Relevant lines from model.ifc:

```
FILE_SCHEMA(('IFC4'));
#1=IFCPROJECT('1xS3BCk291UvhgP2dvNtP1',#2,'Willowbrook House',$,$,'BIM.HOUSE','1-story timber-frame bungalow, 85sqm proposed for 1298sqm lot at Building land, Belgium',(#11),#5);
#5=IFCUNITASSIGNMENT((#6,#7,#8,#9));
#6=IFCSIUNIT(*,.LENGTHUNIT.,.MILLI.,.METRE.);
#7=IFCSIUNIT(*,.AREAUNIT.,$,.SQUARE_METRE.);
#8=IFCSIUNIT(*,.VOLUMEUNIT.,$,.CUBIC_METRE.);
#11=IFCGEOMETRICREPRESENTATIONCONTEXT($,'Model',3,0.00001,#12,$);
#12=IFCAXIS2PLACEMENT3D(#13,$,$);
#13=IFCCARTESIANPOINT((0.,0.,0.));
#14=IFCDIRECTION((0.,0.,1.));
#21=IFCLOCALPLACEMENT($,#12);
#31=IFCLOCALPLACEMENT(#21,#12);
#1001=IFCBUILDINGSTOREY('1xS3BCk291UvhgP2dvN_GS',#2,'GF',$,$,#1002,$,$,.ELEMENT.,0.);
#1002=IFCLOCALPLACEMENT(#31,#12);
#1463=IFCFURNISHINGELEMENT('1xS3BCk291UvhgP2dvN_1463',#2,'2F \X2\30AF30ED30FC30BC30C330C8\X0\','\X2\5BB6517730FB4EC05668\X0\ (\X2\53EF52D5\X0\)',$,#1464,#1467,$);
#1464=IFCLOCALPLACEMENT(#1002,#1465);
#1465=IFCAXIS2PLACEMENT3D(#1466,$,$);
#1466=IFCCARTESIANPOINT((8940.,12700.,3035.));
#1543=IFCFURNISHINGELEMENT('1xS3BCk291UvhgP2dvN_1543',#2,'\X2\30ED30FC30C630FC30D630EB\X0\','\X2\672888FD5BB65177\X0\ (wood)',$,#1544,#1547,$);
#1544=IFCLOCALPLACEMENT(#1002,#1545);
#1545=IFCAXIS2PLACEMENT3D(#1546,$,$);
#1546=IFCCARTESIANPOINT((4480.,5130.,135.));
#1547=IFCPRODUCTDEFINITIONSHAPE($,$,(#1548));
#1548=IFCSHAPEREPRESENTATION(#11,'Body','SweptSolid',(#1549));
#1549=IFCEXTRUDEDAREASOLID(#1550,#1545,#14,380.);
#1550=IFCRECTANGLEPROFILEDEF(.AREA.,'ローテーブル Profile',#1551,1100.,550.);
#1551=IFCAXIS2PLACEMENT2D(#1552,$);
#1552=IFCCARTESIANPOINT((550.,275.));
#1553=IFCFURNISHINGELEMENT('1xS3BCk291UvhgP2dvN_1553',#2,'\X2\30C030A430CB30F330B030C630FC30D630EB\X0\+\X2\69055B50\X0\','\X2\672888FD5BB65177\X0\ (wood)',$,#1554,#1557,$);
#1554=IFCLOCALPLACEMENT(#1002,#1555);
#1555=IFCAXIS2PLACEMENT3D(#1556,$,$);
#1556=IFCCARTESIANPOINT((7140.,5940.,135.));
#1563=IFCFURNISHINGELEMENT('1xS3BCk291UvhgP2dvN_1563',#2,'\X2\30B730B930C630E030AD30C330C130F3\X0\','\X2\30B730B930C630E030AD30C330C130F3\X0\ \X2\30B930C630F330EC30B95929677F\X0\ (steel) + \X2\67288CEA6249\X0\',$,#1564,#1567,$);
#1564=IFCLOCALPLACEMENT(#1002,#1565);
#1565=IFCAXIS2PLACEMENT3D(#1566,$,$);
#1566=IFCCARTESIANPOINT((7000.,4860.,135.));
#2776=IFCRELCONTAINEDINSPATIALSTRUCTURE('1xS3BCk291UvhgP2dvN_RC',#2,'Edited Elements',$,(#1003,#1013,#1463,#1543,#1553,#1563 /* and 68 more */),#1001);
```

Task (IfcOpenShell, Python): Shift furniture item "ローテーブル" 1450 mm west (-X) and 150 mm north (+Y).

```python
import ifcopenshell
import ifcopenshell.api.geometry
import ifcopenshell.util.placement

model = ifcopenshell.open("model.ifc")

item = model.by_guid("1xS3BCk291UvhgP2dvN_1543")
matrix = ifcopenshell.util.placement.get_local_placement(item.ObjectPlacement)
matrix[0, 3] -= 1450.0
matrix[1, 3] += 150.0
ifcopenshell.api.geometry.edit_object_placement(model, product=item, matrix=matrix, is_si=False)

print(ifcopenshell.util.placement.get_local_placement(item.ObjectPlacement).round(3) + 0.0)

model.write("model_rev.ifc")
```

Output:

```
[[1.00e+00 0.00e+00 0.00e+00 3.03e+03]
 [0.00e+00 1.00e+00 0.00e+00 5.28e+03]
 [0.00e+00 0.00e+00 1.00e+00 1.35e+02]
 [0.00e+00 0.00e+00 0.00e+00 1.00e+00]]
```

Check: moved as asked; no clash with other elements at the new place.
